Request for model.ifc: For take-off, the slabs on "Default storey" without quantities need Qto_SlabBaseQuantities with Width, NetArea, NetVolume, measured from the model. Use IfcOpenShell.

First a look at what the model holds.

```python
import ifcopenshell
import ifcopenshell.util.element
import ifcopenshell.util.unit

model = ifcopenshell.open("model.ifc")
print(model.schema)
for unit_type in ("LENGTHUNIT", "AREAUNIT", "VOLUMEUNIT"):
    print(unit_type, ifcopenshell.util.unit.calculate_unit_scale(model, unit_type))
storey = next(s for s in model.by_type("IfcBuildingStorey") if s.Name == "Default storey")
slabs = [e for e in ifcopenshell.util.element.get_decomposition(storey) if e.is_a("IfcSlab")]
for e in sorted(slabs, key=lambda e: e.id()):
    print(e.id(), e.is_a(), e.Name, list(ifcopenshell.util.element.get_psets(e, qtos_only=True)), sep=" | ")
```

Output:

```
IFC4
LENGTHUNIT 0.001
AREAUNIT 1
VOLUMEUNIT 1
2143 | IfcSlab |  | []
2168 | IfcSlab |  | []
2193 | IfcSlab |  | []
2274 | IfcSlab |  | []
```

```python
import ifcopenshell
import ifcopenshell.api.pset
import ifcopenshell.geom
import ifcopenshell.util.element
import ifcopenshell.util.shape
import ifcopenshell.util.unit

model = ifcopenshell.open("model.ifc")
unit_scale = ifcopenshell.util.unit.calculate_unit_scale(model)
area_scale = ifcopenshell.util.unit.calculate_unit_scale(model, "AREAUNIT")
volume_scale = ifcopenshell.util.unit.calculate_unit_scale(model, "VOLUMEUNIT")
settings = ifcopenshell.geom.settings()

storey = next(s for s in model.by_type("IfcBuildingStorey") if s.Name == "Default storey")
slabs = [e for e in ifcopenshell.util.element.get_decomposition(storey) if e.is_a("IfcSlab")]

for e in sorted(slabs, key=lambda e: e.id()):
    if ifcopenshell.util.element.get_psets(e, qtos_only=True, should_inherit=False):
        continue
    # Geometry comes back in metres, in the element's own axes.
    shape = ifcopenshell.geom.create_shape(settings, e)
    values = {
        "Width": ifcopenshell.util.shape.get_z(shape.geometry) / unit_scale,
        "NetArea": ifcopenshell.util.shape.get_footprint_area(shape.geometry) / area_scale,
        "NetVolume": ifcopenshell.util.shape.get_volume(shape.geometry) / volume_scale,
    }
    qto = ifcopenshell.api.pset.add_qto(model, product=e, name="Qto_SlabBaseQuantities")
    ifcopenshell.api.pset.edit_qto(model, qto=qto, properties=values)
    print(e.id(), {k: round(v, 3) for k, v in values.items()})

model.write("model-out.ifc")
```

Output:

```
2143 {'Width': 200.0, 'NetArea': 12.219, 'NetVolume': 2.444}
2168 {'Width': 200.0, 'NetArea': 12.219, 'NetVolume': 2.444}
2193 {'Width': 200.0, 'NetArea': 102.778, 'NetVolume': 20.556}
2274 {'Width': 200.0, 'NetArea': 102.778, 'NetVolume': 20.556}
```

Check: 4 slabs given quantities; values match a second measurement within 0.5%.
